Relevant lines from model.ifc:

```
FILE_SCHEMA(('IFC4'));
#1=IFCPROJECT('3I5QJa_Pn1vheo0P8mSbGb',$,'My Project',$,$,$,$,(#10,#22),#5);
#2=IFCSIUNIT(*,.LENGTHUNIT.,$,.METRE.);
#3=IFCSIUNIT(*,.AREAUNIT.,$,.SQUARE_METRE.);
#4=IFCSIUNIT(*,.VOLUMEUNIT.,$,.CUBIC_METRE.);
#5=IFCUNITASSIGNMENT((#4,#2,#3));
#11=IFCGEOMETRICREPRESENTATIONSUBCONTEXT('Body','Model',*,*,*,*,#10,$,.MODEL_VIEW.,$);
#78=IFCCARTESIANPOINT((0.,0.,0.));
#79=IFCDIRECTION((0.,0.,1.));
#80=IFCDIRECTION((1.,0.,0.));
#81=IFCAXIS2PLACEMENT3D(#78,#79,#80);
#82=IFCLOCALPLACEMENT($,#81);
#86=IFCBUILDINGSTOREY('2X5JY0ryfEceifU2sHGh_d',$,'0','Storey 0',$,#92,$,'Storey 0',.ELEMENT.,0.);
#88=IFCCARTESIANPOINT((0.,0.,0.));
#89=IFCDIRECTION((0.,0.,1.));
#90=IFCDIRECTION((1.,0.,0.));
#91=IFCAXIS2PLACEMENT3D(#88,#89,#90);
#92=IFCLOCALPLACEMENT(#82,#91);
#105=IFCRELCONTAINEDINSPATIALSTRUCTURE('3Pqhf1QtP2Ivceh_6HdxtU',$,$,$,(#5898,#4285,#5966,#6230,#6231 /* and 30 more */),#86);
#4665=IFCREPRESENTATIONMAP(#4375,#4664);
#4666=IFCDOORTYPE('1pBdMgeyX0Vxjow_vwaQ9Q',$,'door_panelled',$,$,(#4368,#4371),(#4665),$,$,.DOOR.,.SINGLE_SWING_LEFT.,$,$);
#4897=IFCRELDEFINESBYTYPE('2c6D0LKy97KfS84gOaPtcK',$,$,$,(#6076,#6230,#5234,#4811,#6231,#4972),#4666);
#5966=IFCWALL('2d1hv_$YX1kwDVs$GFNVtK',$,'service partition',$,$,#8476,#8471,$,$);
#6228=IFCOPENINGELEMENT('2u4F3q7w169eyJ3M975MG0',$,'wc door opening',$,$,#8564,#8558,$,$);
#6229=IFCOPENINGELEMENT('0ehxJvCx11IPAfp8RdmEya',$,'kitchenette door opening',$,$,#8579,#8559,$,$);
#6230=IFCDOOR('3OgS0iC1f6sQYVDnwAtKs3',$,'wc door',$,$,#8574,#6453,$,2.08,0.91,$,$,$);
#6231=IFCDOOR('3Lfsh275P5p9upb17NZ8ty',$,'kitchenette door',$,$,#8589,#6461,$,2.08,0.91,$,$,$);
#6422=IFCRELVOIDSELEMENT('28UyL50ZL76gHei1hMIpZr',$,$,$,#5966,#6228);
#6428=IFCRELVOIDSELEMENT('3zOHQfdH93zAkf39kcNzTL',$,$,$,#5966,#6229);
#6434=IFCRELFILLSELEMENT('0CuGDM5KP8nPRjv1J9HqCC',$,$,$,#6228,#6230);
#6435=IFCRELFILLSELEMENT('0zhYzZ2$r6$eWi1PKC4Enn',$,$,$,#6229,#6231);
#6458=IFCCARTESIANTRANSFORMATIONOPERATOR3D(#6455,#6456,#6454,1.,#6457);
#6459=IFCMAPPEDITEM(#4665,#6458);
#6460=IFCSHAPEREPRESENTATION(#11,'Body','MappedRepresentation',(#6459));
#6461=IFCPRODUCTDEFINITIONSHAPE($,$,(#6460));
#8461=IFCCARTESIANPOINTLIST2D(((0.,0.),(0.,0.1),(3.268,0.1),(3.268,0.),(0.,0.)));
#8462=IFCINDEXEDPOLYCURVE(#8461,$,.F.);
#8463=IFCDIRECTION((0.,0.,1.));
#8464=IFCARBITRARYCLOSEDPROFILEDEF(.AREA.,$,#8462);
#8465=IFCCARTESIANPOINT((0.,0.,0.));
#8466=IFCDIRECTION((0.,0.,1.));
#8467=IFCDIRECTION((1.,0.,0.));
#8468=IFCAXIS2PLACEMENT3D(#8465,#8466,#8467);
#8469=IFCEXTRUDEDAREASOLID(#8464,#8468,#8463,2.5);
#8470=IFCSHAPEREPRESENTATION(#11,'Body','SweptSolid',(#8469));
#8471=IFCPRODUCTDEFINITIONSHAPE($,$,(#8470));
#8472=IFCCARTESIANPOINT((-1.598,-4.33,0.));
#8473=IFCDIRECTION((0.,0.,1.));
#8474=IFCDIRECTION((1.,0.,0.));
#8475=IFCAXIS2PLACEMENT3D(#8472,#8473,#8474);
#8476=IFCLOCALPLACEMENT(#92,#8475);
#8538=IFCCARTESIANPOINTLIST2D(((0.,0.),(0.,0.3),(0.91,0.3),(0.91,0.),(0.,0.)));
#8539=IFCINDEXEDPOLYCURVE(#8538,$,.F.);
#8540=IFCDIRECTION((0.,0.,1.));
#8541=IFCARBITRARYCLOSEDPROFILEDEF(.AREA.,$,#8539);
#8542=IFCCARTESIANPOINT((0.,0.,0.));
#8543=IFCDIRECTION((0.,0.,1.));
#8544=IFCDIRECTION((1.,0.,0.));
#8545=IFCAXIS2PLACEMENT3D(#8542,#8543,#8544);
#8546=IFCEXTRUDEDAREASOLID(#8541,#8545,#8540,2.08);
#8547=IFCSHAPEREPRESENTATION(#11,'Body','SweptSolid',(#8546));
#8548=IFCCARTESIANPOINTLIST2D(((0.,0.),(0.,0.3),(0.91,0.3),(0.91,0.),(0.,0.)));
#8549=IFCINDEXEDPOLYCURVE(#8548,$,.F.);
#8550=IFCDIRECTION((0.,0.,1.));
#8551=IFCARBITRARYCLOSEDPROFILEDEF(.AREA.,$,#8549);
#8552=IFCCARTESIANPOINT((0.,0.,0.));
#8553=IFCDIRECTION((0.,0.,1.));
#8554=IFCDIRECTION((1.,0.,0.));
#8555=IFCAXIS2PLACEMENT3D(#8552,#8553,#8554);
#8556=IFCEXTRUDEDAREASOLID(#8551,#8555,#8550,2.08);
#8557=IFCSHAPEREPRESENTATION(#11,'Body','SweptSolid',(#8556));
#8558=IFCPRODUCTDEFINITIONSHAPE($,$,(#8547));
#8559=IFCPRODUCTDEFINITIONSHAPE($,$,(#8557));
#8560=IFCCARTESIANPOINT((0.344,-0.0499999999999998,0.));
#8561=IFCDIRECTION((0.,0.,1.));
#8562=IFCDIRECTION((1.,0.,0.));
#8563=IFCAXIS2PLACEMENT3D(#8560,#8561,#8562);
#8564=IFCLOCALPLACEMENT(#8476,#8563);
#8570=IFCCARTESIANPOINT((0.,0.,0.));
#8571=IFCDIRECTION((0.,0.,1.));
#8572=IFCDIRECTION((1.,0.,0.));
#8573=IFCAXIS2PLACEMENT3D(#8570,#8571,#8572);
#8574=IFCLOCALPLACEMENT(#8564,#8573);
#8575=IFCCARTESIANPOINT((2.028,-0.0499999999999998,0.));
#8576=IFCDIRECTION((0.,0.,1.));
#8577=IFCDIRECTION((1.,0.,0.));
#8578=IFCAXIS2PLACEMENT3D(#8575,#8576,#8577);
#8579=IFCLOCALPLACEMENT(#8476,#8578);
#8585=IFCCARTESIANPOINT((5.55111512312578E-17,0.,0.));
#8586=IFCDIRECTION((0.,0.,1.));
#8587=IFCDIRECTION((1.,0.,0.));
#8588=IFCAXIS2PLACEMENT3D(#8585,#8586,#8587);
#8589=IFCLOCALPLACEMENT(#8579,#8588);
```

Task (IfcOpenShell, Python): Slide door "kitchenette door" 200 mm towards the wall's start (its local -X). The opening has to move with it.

```python
import ifcopenshell
import ifcopenshell.api.geometry
import ifcopenshell.util.placement

model = ifcopenshell.open("model.ifc")

door = model.by_guid("3Lfsh275P5p9upb17NZ8ty")
opening = door.FillsVoids[0].RelatingOpeningElement
wall = opening.VoidsElements[0].RelatingBuildingElement

wall_matrix = ifcopenshell.util.placement.get_local_placement(wall.ObjectPlacement)
shift = wall_matrix[:3, 0] * -0.2
before = ifcopenshell.util.placement.get_local_placement(door.ObjectPlacement)[:3, 3].copy()

# The door is placed relative to its opening, so it follows when the opening moves.
matrix = ifcopenshell.util.placement.get_local_placement(opening.ObjectPlacement)
matrix[:3, 3] += shift
ifcopenshell.api.geometry.edit_object_placement(
    model, product=opening, matrix=matrix, is_si=False, should_transform_children=True
)

after = ifcopenshell.util.placement.get_local_placement(door.ObjectPlacement)[:3, 3]
print("door moved by", (after - before).round(3) + 0.0)

model.write("model_rev.ifc")
```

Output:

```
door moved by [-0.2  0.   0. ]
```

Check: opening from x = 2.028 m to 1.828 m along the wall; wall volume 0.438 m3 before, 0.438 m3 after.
